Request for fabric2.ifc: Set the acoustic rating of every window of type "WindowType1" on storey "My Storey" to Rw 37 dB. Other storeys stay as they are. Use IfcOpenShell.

First a look at what the model holds.

```python
import ifcopenshell
import ifcopenshell.util.element

model = ifcopenshell.open("fabric2.ifc")
print(model.schema)
storey = next(s for s in model.by_type("IfcBuildingStorey") if s.Name == "My Storey")
windows = [e for e in ifcopenshell.util.element.get_decomposition(storey) if e.is_a("IfcWindow")]
seen = {}
for e in windows:
    element_type = ifcopenshell.util.element.get_type(e)
    key = (element_type.Name if element_type != e and element_type else None, ifcopenshell.util.element.get_pset(e, "Pset_WindowCommon", "AcousticRating"))
    seen[key] = seen.get(key, 0) + 1
for (name, value), count in sorted(seen.items(), key=str):
    print(count, "x", name, "|", value)
```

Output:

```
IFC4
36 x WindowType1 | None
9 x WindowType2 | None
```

```python
import ifcopenshell
import ifcopenshell.api.pset
import ifcopenshell.util.element

model = ifcopenshell.open("fabric2.ifc")

storey = next(s for s in model.by_type("IfcBuildingStorey") if s.Name == "My Storey")
windows = [e for e in ifcopenshell.util.element.get_decomposition(storey) if e.is_a("IfcWindow")]

count = 0
for e in windows:
    element_type = ifcopenshell.util.element.get_type(e)
    if element_type in (None, e) or element_type.Name != "WindowType1":
        continue
    # add_pset returns the element's existing set when there is one.
    pset = ifcopenshell.api.pset.add_pset(model, product=e, name="Pset_WindowCommon")
    ifcopenshell.api.pset.edit_pset(model, pset=pset, properties={"AcousticRating": "Rw 37 dB"})
    count += 1

print(count, "windows updated")

model.write("fabric2-out.ifc")
```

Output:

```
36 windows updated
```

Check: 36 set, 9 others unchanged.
